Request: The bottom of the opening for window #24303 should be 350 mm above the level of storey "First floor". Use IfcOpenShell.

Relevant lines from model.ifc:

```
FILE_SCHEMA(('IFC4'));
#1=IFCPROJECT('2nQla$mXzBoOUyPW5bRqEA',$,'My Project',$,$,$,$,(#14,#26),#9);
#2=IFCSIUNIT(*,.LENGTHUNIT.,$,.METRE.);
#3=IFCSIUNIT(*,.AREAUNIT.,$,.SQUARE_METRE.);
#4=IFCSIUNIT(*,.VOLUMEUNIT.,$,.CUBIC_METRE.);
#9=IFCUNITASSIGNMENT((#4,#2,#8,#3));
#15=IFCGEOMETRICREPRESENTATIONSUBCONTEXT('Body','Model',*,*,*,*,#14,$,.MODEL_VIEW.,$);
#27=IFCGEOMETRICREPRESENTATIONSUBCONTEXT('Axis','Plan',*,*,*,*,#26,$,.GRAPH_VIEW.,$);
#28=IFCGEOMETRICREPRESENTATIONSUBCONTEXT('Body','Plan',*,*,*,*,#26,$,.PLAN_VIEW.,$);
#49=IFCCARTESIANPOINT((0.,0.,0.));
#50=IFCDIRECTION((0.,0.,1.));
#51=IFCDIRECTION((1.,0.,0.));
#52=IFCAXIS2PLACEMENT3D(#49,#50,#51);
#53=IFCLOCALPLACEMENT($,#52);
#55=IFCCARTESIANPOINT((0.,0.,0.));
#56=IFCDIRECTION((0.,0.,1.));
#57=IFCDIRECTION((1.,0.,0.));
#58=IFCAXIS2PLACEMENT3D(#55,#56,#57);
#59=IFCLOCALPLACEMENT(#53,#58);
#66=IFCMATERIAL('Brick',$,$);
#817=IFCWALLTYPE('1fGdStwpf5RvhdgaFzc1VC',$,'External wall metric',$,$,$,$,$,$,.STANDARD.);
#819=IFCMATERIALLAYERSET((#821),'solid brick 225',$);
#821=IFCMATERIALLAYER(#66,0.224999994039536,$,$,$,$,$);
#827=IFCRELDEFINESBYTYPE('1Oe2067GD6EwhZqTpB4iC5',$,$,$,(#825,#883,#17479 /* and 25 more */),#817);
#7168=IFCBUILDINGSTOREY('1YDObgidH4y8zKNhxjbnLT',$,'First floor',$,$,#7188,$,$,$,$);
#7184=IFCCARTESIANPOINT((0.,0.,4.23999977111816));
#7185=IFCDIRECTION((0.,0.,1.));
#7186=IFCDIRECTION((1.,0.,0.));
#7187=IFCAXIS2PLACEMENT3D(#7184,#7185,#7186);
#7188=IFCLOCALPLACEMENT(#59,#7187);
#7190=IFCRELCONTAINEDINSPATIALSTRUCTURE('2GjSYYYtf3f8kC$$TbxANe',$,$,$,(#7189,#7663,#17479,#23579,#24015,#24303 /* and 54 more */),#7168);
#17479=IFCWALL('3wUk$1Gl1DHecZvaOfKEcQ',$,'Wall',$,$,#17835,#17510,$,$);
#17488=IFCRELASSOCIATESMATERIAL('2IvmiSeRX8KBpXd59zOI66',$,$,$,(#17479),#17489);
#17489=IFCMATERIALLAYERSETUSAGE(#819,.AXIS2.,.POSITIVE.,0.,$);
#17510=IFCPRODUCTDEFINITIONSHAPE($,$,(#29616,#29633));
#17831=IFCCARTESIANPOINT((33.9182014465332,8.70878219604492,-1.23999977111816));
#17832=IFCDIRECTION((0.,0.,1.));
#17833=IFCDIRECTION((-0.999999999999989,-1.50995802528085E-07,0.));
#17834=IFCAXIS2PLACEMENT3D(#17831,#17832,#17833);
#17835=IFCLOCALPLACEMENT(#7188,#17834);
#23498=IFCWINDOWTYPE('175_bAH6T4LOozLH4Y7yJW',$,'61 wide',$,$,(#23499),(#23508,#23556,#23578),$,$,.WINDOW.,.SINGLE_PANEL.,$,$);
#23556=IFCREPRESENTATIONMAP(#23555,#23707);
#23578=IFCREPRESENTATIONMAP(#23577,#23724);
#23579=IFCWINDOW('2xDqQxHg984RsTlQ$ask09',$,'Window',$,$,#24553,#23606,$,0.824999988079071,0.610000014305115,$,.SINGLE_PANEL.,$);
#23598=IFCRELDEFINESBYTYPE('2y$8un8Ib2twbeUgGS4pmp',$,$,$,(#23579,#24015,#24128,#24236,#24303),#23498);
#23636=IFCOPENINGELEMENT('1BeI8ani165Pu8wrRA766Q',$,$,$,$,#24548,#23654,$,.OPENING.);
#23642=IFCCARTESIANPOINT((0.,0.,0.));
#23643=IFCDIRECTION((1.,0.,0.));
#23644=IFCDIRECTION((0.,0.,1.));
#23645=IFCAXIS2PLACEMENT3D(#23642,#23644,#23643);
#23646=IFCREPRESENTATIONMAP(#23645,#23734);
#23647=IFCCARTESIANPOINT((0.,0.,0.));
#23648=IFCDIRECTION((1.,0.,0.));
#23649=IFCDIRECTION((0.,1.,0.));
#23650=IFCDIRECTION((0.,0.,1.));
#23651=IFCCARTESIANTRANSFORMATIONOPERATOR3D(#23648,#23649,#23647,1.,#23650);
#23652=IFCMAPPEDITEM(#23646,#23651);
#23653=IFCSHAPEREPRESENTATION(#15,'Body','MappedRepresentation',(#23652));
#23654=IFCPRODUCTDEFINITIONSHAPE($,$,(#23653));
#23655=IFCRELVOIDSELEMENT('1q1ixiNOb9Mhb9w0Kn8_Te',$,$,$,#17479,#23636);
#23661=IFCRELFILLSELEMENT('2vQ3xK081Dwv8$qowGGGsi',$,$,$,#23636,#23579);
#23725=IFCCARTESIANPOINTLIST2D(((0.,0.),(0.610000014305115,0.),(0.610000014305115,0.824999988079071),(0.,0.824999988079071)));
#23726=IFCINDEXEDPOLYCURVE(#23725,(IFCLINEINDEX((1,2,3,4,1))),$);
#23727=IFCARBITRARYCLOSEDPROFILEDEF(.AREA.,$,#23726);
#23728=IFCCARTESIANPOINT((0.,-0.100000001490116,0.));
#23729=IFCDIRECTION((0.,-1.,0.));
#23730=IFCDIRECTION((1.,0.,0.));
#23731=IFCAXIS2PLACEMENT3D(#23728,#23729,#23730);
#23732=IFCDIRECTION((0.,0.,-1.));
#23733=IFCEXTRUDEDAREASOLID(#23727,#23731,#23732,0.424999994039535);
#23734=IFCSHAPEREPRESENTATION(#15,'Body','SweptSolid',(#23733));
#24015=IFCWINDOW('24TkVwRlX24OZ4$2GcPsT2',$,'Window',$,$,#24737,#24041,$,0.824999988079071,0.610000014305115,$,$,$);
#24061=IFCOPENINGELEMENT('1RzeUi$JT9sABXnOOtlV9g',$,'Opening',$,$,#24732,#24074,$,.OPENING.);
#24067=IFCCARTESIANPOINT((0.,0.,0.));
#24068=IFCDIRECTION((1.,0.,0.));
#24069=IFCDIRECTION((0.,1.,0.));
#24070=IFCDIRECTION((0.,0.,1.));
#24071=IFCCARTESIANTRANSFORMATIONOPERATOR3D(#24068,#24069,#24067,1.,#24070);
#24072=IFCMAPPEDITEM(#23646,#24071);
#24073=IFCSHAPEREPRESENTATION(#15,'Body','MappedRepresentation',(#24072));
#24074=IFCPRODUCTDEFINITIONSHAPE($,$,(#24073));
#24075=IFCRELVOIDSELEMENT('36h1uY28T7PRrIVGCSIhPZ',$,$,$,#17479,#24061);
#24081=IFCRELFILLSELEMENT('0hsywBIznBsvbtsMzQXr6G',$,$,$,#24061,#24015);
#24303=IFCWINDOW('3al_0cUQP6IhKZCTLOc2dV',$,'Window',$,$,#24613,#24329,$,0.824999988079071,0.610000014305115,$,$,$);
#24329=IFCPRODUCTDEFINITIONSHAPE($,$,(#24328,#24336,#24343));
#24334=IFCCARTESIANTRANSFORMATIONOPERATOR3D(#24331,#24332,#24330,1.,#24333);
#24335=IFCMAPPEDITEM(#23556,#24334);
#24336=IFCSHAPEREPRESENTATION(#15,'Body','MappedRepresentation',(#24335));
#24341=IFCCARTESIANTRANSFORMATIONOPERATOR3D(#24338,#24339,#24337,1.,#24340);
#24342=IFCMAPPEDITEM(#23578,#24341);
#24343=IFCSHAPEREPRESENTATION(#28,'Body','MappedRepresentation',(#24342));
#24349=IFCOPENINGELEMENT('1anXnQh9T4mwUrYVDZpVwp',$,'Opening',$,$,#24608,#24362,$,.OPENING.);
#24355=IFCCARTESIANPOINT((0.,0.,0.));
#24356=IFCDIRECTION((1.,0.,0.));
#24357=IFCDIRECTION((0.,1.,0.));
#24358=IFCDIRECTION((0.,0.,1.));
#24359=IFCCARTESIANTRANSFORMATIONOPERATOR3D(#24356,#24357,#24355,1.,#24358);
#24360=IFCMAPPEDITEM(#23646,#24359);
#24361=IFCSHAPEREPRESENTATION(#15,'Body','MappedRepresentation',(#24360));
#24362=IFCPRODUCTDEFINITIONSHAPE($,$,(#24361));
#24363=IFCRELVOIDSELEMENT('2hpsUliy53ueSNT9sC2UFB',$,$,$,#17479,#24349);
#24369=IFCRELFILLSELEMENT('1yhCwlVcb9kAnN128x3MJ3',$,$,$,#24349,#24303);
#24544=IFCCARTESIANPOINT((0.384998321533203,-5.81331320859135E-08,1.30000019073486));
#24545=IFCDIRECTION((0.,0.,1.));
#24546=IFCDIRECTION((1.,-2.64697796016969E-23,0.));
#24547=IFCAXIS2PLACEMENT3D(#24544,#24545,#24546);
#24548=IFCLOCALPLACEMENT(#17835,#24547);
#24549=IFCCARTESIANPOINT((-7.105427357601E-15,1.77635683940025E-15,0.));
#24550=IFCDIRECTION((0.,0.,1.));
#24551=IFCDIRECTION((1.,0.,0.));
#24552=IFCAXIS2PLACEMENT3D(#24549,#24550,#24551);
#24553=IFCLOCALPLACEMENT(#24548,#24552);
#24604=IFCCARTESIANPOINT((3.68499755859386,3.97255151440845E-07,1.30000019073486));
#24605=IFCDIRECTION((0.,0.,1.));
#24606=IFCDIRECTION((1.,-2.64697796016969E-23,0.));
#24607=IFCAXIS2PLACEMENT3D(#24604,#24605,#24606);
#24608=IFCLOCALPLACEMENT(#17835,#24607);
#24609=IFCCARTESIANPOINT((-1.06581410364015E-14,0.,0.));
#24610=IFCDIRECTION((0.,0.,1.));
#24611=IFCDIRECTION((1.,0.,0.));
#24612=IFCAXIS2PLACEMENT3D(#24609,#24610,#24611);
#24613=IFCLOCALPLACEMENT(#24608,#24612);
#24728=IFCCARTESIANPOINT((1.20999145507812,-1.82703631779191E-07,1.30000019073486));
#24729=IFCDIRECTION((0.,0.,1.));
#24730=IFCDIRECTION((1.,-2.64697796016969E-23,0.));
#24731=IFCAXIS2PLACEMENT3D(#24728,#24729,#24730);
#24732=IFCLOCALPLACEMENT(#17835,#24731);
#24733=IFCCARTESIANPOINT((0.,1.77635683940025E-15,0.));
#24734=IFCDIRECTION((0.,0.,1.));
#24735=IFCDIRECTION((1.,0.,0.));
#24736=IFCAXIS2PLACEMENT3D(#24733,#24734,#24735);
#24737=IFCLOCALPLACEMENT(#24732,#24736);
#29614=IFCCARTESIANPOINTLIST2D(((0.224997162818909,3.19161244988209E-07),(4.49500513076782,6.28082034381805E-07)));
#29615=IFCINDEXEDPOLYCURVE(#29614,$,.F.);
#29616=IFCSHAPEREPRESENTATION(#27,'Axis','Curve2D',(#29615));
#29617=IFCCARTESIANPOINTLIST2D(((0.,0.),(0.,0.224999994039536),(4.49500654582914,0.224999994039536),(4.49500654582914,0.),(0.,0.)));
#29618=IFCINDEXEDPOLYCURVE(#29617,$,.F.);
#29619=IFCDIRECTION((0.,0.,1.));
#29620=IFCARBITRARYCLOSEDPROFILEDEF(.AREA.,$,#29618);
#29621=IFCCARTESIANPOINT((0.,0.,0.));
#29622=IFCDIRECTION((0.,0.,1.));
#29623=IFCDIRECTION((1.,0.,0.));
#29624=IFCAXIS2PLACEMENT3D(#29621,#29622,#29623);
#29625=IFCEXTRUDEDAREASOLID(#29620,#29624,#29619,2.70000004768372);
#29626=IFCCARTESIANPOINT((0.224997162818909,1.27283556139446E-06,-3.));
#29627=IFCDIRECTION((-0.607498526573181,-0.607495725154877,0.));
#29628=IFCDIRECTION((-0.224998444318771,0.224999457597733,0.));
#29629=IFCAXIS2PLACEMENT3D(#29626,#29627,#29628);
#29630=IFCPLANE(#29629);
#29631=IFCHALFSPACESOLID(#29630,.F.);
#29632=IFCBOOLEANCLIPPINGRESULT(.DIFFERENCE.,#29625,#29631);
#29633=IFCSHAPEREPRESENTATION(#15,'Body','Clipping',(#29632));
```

```python
import numpy as np
import ifcopenshell
import ifcopenshell.api.geometry
import ifcopenshell.geom
import ifcopenshell.util.element
import ifcopenshell.util.placement
import ifcopenshell.util.shape
import ifcopenshell.util.unit

model = ifcopenshell.open("model.ifc")
unit_scale = ifcopenshell.util.unit.calculate_unit_scale(model)

window = model.by_guid("3al_0cUQP6IhKZCTLOc2dV")
opening = window.FillsVoids[0].RelatingOpeningElement
storey = ifcopenshell.util.element.get_container(window, ifc_class="IfcBuildingStorey")
level = ifcopenshell.util.placement.get_local_placement(storey.ObjectPlacement)[2, 3]

# The opening's origin need not be at the sill, so measure its lowest point.
shape = ifcopenshell.geom.create_shape(ifcopenshell.geom.settings(), opening)
bottom = ifcopenshell.util.shape.get_shape_bottom_elevation(shape, shape.geometry) / unit_scale
dz = level + 0.35 / unit_scale - bottom

shift = np.array([0.0, 0.0, dz])
# The window is placed relative to its opening, so it follows when the opening moves.
matrix = ifcopenshell.util.placement.get_local_placement(opening.ObjectPlacement)
matrix[:3, 3] += shift
ifcopenshell.api.geometry.edit_object_placement(
    model, product=opening, matrix=matrix, is_si=False, should_transform_children=True
)

print(f"moved by {dz * unit_scale:+.3f} m")

model.write("model_v2.ifc")
```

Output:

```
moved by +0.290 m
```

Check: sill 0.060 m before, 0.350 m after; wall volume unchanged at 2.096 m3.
